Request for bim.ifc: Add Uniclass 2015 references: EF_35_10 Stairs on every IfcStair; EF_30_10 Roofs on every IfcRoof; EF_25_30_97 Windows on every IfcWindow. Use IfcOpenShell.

First a look at what the model holds.

```python
import ifcopenshell

model = ifcopenshell.open("bim.ifc")
print(model.schema)
print("classifications:", [c.Name for c in model.by_type("IfcClassification")])
for ifc_class in ("IfcDoor", "IfcRoof", "IfcStair", "IfcWall", "IfcWindow"):
    print(ifc_class, len(model.by_type(ifc_class)))
```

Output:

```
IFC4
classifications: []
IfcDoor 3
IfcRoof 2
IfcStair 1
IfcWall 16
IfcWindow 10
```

```python
import ifcopenshell
import ifcopenshell.api.classification

model = ifcopenshell.open("bim.ifc")

system = ifcopenshell.api.classification.add_classification(model, classification="Uniclass 2015")

codes = {
    "IfcStair": ("EF_35_10", "Stairs"),
    "IfcRoof": ("EF_30_10", "Roofs"),
    "IfcWindow": ("EF_25_30_97", "Windows"),
}
for ifc_class, (code, name) in codes.items():
    products = model.by_type(ifc_class)
    ifcopenshell.api.classification.add_reference(
        model, products=products, classification=system, identification=code, name=name
    )
    print(code, len(products))

model.write("bim_updated.ifc")
```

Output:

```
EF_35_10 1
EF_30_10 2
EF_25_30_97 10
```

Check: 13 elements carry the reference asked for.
